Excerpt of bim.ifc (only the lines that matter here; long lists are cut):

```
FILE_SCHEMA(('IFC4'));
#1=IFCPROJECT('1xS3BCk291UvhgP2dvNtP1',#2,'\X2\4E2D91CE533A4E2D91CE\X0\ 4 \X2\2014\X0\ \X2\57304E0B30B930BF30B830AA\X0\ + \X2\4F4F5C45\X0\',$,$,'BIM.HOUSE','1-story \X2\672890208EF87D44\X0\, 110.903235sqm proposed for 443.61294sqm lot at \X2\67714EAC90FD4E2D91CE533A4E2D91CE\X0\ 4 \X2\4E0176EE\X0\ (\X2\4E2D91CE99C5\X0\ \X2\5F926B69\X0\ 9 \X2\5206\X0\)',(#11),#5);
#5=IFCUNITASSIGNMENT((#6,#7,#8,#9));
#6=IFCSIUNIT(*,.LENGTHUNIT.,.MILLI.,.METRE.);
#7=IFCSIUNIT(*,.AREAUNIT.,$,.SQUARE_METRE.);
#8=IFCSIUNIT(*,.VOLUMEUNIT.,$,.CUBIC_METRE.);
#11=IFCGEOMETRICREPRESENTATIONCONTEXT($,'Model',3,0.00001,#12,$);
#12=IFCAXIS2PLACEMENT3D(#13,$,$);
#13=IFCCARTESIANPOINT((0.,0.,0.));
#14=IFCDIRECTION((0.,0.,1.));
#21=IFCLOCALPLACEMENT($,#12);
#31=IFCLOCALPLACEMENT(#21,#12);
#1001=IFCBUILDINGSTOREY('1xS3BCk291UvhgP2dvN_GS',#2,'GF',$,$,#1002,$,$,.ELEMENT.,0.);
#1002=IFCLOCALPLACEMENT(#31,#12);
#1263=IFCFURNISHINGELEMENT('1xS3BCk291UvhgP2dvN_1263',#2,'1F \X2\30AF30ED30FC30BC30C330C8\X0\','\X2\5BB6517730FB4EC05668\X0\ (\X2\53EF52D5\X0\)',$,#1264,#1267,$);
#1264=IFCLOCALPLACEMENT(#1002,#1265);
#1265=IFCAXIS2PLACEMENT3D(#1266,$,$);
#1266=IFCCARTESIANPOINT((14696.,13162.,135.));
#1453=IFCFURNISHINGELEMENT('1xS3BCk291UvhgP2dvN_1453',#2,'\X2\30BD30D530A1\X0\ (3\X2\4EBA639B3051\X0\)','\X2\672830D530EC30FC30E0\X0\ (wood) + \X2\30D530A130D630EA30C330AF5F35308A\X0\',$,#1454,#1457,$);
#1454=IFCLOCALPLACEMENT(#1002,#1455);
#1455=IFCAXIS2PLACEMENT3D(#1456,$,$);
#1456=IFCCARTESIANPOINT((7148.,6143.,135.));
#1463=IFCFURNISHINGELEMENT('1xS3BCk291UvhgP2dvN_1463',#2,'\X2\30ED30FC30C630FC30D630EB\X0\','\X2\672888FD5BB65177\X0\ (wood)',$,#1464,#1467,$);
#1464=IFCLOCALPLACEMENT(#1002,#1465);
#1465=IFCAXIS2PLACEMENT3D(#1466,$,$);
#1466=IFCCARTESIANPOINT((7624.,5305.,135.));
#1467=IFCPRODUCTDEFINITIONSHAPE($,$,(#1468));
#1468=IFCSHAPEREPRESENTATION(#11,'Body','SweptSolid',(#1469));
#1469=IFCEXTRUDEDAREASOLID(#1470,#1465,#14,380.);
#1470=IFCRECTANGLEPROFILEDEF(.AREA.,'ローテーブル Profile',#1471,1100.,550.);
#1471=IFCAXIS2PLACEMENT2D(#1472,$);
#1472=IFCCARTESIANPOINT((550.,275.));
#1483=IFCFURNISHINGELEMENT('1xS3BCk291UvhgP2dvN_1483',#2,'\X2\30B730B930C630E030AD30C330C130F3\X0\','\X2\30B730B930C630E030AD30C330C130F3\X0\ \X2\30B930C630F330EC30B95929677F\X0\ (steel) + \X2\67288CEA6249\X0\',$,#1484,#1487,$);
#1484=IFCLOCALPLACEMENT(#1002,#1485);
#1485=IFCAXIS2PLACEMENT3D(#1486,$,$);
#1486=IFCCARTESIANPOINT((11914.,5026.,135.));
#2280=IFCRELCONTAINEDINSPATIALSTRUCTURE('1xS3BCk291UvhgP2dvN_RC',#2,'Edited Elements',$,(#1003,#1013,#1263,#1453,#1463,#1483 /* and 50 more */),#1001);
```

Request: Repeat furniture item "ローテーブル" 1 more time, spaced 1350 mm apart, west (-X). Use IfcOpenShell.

```python
import numpy as np
import ifcopenshell
import ifcopenshell.api.geometry
import ifcopenshell.api.root
import ifcopenshell.util.element
import ifcopenshell.util.placement

model = ifcopenshell.open("bim.ifc")


def reuse_history(source, copy):
    """copy_class also copies each property set's owner history, people and application; keep the originals."""
    for rel in copy.IsDefinedBy:
        if rel.is_a("IfcRelDefinesByProperties") and (history := rel.RelatingPropertyDefinition.OwnerHistory):
            rel.RelatingPropertyDefinition.OwnerHistory = source.OwnerHistory
            ifcopenshell.util.element.remove_deep2(model, history)


source = model.by_guid("1xS3BCk291UvhgP2dvN_1463")
base = ifcopenshell.util.placement.get_local_placement(source.ObjectPlacement)
step = np.array([-1.0, 0.0, 0.0]) * 1350.0

for i in range(1, 2):
    copy = ifcopenshell.api.root.copy_class(model, product=source)
    copy.Representation = ifcopenshell.util.element.copy_deep(
        model, source.Representation, exclude=["IfcGeometricRepresentationContext", "IfcRepresentationMap"]
    )
    reuse_history(source, copy)
    matrix = base.copy()
    matrix[:3, 3] += i * step
    print("added at", matrix[:3, 3].round(3) + 0.0)
    ifcopenshell.api.geometry.edit_object_placement(model, product=copy, matrix=matrix, is_si=False)

model.write("bim-out.ifc")
```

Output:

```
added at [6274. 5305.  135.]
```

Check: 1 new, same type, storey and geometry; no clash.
